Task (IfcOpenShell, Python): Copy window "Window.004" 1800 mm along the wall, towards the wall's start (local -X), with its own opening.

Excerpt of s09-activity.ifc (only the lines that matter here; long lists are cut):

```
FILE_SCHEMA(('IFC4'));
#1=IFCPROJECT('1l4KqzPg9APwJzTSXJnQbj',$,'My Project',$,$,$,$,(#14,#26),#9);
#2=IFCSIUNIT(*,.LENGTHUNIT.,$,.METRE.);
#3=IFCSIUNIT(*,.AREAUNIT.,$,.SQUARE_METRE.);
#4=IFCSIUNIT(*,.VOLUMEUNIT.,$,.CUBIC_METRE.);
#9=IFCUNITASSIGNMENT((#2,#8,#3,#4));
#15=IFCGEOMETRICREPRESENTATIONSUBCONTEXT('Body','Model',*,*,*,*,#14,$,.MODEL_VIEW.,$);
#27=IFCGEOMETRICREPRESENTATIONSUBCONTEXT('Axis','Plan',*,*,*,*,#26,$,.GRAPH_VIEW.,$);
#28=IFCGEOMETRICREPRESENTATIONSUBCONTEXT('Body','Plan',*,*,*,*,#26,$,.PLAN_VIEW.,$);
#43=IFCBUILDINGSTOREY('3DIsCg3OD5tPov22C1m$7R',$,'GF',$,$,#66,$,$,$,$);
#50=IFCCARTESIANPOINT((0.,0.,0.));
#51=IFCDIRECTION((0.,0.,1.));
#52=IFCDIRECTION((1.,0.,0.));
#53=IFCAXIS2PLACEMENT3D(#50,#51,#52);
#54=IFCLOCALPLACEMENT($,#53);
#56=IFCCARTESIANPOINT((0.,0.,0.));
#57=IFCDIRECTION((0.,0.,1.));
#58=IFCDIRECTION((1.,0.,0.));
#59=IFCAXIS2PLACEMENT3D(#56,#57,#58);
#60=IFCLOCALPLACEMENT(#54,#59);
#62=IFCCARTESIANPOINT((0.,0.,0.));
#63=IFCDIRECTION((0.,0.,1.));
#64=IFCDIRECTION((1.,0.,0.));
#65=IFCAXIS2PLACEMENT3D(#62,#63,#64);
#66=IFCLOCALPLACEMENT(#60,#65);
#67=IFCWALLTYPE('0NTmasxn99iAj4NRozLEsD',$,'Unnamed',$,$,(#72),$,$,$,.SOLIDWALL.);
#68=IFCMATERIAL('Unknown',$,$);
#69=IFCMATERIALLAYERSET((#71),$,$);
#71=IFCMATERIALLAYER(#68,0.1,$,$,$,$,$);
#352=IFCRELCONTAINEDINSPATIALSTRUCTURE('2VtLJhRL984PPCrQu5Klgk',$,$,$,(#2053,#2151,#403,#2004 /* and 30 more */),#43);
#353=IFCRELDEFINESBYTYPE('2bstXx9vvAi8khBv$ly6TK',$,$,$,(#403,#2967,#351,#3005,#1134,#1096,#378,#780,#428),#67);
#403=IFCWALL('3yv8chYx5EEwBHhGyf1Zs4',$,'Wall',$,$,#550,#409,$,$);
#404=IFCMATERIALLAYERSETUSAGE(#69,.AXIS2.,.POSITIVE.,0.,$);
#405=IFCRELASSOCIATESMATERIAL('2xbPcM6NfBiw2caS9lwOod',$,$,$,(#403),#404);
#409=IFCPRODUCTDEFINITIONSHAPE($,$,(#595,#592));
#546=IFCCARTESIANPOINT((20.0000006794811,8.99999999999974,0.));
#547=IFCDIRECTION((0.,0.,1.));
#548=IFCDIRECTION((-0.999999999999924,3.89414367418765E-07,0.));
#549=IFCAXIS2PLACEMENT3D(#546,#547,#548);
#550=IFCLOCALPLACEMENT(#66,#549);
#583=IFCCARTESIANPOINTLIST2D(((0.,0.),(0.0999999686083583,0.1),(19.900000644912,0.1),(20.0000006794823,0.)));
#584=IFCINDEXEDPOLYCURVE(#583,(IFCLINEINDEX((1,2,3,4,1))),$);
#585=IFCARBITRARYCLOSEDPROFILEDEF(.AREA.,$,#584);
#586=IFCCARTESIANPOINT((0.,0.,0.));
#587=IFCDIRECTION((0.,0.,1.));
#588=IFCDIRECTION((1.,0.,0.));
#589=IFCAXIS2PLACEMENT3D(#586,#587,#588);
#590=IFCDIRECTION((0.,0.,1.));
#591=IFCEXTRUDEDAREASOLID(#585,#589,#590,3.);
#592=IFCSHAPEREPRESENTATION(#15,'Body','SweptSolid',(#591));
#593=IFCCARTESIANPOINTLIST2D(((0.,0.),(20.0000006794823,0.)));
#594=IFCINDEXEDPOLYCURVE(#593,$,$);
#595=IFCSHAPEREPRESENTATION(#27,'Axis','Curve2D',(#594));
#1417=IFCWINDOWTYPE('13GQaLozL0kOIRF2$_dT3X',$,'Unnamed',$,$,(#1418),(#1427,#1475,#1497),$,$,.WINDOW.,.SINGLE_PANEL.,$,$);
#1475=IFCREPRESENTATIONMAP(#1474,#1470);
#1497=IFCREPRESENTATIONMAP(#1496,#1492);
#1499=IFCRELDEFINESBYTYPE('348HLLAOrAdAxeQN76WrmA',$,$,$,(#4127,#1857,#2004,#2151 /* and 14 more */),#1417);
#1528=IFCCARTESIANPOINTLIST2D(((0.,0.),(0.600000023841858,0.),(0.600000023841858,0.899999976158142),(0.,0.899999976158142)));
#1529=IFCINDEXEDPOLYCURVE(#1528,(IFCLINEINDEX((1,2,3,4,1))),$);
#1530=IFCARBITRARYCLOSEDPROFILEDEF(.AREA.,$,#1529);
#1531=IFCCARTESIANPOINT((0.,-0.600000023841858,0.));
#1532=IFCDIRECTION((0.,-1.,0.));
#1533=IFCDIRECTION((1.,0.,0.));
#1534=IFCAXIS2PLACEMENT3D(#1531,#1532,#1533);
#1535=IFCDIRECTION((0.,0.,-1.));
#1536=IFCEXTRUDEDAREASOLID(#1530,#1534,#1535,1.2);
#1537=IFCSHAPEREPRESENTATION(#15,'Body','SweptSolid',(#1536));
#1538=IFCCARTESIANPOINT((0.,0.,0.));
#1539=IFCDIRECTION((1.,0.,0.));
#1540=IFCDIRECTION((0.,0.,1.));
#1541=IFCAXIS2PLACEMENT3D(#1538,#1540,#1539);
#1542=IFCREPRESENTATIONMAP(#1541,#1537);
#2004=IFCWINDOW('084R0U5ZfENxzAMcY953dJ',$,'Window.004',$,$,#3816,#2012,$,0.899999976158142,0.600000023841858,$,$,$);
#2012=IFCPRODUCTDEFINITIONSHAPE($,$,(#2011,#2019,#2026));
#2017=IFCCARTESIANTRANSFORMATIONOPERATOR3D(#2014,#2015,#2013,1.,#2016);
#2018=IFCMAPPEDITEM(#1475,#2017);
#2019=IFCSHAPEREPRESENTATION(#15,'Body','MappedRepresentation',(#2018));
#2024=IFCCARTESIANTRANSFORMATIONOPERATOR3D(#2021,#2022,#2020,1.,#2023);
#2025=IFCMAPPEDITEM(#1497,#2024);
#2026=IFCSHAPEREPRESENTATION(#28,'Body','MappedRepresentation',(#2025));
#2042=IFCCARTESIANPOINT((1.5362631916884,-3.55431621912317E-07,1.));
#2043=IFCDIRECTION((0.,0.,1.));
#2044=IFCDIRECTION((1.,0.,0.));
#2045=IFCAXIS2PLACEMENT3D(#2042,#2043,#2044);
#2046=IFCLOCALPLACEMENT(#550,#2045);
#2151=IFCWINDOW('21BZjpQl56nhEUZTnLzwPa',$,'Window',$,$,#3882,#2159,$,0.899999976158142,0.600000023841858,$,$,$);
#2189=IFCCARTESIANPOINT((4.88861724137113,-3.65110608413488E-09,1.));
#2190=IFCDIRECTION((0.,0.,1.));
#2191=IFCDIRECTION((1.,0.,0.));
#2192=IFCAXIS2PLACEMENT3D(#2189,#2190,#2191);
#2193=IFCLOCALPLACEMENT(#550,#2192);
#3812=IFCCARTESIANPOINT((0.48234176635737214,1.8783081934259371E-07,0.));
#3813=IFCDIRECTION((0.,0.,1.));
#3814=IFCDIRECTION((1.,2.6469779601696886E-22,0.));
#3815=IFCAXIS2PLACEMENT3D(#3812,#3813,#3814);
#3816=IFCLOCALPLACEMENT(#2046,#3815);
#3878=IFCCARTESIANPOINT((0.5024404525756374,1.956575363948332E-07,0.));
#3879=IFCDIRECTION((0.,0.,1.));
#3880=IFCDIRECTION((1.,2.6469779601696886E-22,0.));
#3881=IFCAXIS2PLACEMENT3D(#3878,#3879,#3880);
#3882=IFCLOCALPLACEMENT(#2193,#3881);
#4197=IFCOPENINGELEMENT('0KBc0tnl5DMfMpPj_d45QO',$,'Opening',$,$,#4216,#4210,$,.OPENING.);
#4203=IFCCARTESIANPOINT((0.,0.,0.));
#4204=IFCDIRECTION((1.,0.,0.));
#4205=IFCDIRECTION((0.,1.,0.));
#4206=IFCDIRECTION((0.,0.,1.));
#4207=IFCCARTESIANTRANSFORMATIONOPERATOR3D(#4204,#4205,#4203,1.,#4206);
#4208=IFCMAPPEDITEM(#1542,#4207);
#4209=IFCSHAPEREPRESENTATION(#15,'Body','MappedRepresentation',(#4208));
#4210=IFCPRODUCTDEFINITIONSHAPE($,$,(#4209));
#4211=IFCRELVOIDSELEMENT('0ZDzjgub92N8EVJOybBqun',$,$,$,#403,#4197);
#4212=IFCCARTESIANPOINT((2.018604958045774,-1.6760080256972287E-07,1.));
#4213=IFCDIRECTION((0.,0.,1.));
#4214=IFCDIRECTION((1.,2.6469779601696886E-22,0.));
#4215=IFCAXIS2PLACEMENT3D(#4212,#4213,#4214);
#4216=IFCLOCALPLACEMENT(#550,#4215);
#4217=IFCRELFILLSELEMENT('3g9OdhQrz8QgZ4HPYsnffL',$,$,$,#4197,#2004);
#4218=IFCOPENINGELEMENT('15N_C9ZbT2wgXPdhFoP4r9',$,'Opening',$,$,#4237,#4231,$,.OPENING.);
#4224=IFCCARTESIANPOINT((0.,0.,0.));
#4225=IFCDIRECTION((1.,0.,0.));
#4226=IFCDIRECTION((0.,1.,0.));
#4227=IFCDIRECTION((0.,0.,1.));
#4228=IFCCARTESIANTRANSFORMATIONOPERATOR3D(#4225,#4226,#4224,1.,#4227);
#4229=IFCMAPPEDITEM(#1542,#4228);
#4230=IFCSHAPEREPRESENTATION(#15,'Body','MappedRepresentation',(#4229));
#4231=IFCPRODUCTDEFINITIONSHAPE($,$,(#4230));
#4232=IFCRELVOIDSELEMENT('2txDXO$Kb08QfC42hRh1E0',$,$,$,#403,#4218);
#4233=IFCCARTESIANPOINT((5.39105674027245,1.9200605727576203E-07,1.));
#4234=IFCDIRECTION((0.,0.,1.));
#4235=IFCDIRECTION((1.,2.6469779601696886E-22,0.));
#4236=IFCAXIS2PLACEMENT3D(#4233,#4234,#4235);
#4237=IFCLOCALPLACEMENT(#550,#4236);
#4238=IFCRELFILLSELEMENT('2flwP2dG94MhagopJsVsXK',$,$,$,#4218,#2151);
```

```python
import ifcopenshell
import ifcopenshell.api.feature
import ifcopenshell.api.geometry
import ifcopenshell.api.root
import ifcopenshell.geom
import ifcopenshell.util.element
import ifcopenshell.util.placement
import ifcopenshell.util.shape
import ifcopenshell.util.unit

model = ifcopenshell.open("s09-activity.ifc")
unit_scale = ifcopenshell.util.unit.calculate_unit_scale(model)
settings = ifcopenshell.geom.settings()


def volume(element):
    """Net volume in cubic metres, openings subtracted."""
    shape = ifcopenshell.geom.create_shape(settings, element)
    return ifcopenshell.util.shape.get_volume(shape.geometry)


window = model.by_id(2004)
opening = window.FillsVoids[0].RelatingOpeningElement
wall = opening.VoidsElements[0].RelatingBuildingElement
before = volume(wall)
shift = ifcopenshell.util.placement.get_local_placement(wall.ObjectPlacement)[:3, 0] * -1.8 / unit_scale

# copy_class copies the void relationship, type, container and properties, but no geometry.
new_opening = ifcopenshell.api.root.copy_class(model, product=opening)
new_opening.Representation = ifcopenshell.util.element.copy_deep(
    model, opening.Representation, exclude=["IfcGeometricRepresentationContext", "IfcRepresentationMap"]
)
new_window = ifcopenshell.api.root.copy_class(model, product=window)
new_window.Representation = ifcopenshell.util.element.copy_deep(
    model, window.Representation, exclude=["IfcGeometricRepresentationContext", "IfcRepresentationMap"]
)
ifcopenshell.api.feature.add_filling(model, opening=new_opening, element=new_window)

for old, new in ((opening, new_opening), (window, new_window)):
    matrix = ifcopenshell.util.placement.get_local_placement(old.ObjectPlacement)
    matrix[:3, 3] += shift
    ifcopenshell.api.geometry.edit_object_placement(model, product=new, matrix=matrix, is_si=False)

after = volume(wall)

print(f"wall volume {before:.3f} -> {after:.3f} m3")

model.write("s09-activity_updated.ifc")
```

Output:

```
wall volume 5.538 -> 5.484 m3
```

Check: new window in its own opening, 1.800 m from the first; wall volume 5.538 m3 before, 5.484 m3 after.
